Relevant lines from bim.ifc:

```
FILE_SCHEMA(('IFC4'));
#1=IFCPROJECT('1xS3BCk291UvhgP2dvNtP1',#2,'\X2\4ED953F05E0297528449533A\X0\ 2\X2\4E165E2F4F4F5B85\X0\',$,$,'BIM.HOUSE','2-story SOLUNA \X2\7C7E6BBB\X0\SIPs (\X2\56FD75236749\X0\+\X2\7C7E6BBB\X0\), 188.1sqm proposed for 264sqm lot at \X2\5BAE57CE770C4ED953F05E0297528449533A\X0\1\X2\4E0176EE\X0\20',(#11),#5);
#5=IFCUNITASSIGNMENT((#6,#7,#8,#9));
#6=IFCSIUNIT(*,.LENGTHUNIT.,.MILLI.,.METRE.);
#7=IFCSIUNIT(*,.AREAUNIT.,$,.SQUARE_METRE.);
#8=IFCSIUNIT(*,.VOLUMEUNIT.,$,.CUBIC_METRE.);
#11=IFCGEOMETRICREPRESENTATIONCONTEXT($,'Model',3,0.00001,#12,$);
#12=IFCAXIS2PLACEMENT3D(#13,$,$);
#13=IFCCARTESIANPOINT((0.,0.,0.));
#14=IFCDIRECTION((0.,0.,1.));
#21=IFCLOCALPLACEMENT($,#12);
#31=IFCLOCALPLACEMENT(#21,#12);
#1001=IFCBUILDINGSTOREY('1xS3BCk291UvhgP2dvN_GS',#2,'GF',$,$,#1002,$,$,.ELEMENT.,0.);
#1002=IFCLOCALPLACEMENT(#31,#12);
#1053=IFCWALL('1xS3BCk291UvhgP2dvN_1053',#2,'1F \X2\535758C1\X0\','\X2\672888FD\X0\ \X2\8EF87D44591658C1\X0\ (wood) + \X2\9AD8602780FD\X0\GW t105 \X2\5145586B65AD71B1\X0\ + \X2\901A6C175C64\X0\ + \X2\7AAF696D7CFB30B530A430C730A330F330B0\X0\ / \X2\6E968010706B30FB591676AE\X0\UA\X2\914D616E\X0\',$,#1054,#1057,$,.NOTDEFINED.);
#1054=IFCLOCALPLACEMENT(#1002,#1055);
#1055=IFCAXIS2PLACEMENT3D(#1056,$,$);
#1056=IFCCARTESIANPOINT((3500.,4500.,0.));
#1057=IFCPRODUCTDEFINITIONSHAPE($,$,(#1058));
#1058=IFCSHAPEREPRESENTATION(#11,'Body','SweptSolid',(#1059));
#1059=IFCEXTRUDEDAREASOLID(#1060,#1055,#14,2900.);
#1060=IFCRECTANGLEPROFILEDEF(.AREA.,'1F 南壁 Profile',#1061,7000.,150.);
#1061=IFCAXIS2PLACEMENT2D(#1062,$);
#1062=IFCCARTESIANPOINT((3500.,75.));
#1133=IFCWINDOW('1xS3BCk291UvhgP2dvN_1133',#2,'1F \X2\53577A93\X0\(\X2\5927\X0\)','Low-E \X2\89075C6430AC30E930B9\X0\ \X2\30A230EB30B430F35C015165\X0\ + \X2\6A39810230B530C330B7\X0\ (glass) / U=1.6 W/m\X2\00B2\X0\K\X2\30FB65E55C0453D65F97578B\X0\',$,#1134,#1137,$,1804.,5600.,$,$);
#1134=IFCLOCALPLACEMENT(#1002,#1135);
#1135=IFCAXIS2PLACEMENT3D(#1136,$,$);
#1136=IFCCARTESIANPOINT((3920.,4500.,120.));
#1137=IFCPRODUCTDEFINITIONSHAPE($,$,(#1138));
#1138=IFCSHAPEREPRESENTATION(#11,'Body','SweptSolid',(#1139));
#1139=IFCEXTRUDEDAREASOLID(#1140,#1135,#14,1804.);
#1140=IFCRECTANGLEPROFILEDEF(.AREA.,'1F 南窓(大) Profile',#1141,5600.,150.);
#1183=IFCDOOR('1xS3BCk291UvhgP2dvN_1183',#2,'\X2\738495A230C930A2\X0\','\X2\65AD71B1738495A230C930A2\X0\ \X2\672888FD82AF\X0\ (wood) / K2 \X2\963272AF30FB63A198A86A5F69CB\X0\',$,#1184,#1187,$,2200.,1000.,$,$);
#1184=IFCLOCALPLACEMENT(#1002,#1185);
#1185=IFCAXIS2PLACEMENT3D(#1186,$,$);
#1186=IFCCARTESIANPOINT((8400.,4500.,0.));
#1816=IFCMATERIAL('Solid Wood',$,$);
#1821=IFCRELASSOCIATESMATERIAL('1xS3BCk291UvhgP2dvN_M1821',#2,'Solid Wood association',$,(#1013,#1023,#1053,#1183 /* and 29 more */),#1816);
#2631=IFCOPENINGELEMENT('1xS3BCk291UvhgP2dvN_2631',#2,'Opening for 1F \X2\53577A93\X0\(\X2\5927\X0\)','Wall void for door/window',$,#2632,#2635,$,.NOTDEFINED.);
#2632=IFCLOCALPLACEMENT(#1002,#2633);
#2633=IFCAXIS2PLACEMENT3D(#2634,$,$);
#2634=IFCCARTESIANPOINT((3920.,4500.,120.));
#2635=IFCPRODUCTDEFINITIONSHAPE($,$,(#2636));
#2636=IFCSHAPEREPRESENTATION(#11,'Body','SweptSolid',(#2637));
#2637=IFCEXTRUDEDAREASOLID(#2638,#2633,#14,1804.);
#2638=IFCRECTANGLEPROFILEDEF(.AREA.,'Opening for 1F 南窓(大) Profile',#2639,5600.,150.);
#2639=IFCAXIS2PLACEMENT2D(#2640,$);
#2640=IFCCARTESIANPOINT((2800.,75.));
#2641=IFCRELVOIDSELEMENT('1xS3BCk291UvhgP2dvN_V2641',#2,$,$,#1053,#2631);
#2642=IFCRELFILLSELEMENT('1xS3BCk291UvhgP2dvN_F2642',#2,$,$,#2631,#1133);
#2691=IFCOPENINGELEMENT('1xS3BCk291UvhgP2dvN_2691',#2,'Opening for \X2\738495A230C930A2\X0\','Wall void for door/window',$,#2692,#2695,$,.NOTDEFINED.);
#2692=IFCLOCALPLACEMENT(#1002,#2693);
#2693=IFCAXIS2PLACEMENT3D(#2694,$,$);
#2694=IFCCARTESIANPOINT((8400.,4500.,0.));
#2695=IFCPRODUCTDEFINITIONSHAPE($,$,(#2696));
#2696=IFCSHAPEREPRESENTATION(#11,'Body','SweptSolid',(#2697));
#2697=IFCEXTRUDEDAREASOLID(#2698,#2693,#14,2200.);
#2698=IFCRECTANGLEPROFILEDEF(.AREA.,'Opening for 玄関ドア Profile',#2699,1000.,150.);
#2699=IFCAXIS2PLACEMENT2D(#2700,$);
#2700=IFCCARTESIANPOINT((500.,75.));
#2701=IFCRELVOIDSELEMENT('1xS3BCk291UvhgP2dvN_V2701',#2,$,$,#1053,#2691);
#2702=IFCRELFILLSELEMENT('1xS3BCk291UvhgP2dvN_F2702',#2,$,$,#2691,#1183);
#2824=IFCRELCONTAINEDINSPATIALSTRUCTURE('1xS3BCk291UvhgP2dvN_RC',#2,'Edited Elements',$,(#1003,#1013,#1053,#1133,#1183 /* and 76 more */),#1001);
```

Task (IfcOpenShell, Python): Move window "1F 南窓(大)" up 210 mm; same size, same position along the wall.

```python
import numpy as np
import ifcopenshell
import ifcopenshell.api.geometry
import ifcopenshell.util.placement
import ifcopenshell.util.unit

model = ifcopenshell.open("bim.ifc")
unit_scale = ifcopenshell.util.unit.calculate_unit_scale(model)

window = model.by_id(1133)
opening = window.FillsVoids[0].RelatingOpeningElement
dz = 210.0

shift = np.array([0.0, 0.0, dz])
# The window is not placed relative to its opening, so move both.
for product in (opening, window):
    matrix = ifcopenshell.util.placement.get_local_placement(product.ObjectPlacement)
    matrix[:3, 3] += shift
    ifcopenshell.api.geometry.edit_object_placement(model, product=product, matrix=matrix, is_si=False)

print(f"moved by {dz * unit_scale:+.3f} m")

model.write("bim-out.ifc")
```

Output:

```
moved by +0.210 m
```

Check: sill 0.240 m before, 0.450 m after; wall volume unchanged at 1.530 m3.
